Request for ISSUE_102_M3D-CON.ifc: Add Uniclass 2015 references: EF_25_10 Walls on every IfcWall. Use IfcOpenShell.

First a look at what the model holds.

```python
import ifcopenshell

model = ifcopenshell.open("ISSUE_102_M3D-CON.ifc")
print(model.schema)
print("classifications:", [c.Name for c in model.by_type("IfcClassification")])
for ifc_class in ("IfcDoor", "IfcRoof", "IfcStair", "IfcWall", "IfcWindow"):
    print(ifc_class, len(model.by_type(ifc_class)))
```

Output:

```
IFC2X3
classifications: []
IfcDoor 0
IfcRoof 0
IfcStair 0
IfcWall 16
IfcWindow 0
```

```python
import ifcopenshell
import ifcopenshell.api.classification

model = ifcopenshell.open("ISSUE_102_M3D-CON.ifc")

# IFC2X3 requires Source and Edition and has no link from the project to the system.
system = model.create_entity("IfcClassification", Source="NBS", Edition="2015", Name="Uniclass 2015")

codes = {
    "IfcWall": ("EF_25_10", "Walls"),
}
for ifc_class, (code, name) in codes.items():
    products = model.by_type(ifc_class)
    ifcopenshell.api.classification.add_reference(
        model, products=products, classification=system, identification=code, name=name
    )
    print(code, len(products))

model.write("ISSUE_102_M3D-CON_rev.ifc")
```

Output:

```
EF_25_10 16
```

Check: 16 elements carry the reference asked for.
